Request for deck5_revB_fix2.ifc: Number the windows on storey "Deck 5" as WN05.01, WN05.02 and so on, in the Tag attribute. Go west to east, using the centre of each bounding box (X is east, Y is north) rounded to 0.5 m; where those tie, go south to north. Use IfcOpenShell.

First a look at what the model holds.

```python
import ifcopenshell
import ifcopenshell.util.element
import ifcopenshell.util.placement

model = ifcopenshell.open("deck5_revB_fix2.ifc")
print(model.schema)
storey = next(s for s in model.by_type("IfcBuildingStorey") if s.Name == "Deck 5")
windows = [e for e in ifcopenshell.util.element.get_decomposition(storey) if e.is_a("IfcWindow")]
for e in sorted(windows, key=lambda e: e.id()):
    origin = ifcopenshell.util.placement.get_local_placement(e.ObjectPlacement)[:3, 3]
    print(e.id(), e.Tag, e.Name, origin.round(2) + 0.0, sep=" | ")
```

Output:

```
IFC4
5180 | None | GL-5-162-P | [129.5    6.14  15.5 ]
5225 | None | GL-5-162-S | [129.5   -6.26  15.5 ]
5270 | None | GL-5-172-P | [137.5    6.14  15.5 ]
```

```python
import ifcopenshell
import ifcopenshell.geom
import ifcopenshell.util.element
import ifcopenshell.util.shape

model = ifcopenshell.open("deck5_revB_fix2.ifc")
settings = ifcopenshell.geom.settings()
settings.set("use-world-coords", True)


def centre(element):
    shape = ifcopenshell.geom.create_shape(settings, element)
    return ifcopenshell.util.shape.get_bbox_centroid(shape.geometry)


storey = next(s for s in model.by_type("IfcBuildingStorey") if s.Name == "Deck 5")
windows = [e for e in ifcopenshell.util.element.get_decomposition(storey) if e.is_a("IfcWindow")]

# Insertion points can sit at a corner or the storey origin, so sort by the geometry (in metres).
centres = {e: centre(e) for e in windows}
windows.sort(key=lambda e: (round(centres[e][0] / 0.5), centres[e][1]))

for i, e in enumerate(windows, start=1):
    number = f"WN05.{i:02d}"
    e.Tag = number
    print(e.id(), number)

model.write("deck5_revB_fix2-out.ifc")
```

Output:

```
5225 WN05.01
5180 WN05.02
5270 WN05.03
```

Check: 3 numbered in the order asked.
